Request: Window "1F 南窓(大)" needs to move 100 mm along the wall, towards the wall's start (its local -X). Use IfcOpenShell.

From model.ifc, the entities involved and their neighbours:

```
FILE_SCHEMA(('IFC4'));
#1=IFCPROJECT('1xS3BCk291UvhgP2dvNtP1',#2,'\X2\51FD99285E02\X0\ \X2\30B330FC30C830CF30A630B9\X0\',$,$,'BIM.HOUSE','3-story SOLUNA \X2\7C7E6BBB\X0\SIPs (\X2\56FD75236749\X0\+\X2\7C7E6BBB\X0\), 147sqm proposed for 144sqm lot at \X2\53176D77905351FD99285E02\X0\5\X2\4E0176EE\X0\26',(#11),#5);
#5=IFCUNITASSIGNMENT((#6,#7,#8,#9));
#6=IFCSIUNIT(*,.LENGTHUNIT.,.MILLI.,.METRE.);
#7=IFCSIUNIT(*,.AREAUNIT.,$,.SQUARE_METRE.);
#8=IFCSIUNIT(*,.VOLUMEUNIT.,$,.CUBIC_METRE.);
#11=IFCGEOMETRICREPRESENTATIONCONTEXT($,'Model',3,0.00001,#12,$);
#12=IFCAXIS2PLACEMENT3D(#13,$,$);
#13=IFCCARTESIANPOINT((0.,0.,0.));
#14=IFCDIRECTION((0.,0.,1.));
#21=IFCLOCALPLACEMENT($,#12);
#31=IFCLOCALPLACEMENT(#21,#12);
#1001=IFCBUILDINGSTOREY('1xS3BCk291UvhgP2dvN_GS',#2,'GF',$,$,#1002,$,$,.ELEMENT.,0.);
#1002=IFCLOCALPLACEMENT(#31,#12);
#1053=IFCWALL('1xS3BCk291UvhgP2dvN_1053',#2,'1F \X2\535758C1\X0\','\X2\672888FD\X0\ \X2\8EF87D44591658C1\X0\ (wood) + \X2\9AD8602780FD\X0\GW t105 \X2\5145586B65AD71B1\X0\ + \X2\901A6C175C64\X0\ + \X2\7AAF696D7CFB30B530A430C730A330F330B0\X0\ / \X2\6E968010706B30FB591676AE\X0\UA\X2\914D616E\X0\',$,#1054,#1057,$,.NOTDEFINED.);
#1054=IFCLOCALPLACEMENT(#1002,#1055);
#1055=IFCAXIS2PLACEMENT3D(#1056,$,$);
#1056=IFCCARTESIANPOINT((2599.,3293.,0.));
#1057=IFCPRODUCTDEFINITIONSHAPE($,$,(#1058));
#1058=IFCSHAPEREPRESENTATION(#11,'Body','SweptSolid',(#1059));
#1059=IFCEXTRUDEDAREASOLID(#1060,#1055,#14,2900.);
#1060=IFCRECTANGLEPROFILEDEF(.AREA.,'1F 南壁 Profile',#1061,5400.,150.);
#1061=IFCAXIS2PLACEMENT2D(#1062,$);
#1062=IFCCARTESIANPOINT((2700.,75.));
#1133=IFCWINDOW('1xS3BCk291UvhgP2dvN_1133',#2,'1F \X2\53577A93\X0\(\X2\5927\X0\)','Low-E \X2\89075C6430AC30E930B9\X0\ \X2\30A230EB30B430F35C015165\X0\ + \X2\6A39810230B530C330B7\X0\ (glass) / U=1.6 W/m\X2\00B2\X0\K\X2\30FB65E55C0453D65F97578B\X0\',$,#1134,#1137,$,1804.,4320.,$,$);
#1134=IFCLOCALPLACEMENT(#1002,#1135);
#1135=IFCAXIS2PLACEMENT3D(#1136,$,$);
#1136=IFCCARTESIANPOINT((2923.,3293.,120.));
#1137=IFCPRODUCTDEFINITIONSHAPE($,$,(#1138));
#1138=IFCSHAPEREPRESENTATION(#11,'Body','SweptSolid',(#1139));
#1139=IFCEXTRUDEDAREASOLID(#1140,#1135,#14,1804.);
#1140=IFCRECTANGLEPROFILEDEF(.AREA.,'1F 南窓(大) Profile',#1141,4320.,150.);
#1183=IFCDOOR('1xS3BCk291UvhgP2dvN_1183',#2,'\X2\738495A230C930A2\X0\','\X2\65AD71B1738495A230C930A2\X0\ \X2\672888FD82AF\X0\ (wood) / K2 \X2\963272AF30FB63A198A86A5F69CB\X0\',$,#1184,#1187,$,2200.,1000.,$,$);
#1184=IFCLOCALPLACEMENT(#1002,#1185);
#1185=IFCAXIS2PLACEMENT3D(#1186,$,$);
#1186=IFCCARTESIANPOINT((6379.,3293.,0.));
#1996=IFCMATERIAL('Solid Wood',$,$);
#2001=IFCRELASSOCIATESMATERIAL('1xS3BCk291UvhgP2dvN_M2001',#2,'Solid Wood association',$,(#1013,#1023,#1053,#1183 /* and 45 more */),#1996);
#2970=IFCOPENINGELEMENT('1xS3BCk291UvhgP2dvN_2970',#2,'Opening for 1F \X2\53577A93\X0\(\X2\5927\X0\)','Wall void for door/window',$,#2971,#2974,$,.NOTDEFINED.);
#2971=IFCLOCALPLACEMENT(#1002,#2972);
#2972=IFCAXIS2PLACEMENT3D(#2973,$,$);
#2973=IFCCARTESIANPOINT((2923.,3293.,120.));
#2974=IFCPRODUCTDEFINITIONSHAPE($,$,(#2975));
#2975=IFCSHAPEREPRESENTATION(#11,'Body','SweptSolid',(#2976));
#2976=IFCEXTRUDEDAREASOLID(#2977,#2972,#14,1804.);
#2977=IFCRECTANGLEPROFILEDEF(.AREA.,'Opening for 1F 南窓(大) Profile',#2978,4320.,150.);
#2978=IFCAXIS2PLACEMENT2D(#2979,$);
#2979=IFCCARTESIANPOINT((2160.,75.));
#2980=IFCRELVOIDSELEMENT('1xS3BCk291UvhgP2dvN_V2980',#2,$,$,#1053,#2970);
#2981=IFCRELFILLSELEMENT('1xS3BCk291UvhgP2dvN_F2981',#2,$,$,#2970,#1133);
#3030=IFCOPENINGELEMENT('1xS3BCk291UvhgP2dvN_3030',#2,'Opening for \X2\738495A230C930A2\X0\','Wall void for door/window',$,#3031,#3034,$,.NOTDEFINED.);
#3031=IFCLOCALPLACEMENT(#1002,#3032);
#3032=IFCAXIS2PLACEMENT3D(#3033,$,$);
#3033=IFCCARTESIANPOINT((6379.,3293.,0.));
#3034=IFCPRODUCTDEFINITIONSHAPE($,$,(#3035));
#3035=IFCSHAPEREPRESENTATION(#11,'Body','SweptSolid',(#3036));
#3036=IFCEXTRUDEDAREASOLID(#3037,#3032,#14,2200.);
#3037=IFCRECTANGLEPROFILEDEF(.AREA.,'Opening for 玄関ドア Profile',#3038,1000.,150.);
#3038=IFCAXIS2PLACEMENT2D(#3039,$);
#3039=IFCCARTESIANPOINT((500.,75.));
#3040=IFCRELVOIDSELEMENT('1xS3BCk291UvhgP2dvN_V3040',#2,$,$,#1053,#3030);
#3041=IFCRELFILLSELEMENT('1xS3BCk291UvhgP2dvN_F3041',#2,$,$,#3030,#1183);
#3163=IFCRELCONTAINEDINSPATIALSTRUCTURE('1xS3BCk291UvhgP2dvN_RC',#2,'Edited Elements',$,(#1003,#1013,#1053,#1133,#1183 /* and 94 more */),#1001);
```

```python
import ifcopenshell
import ifcopenshell.api.geometry
import ifcopenshell.util.placement
import ifcopenshell.util.unit

model = ifcopenshell.open("model.ifc")
unit_scale = ifcopenshell.util.unit.calculate_unit_scale(model)

window = model.by_guid("1xS3BCk291UvhgP2dvN_1133")
opening = window.FillsVoids[0].RelatingOpeningElement
wall = opening.VoidsElements[0].RelatingBuildingElement

wall_matrix = ifcopenshell.util.placement.get_local_placement(wall.ObjectPlacement)
shift = wall_matrix[:3, 0] * -0.1 / unit_scale
before = ifcopenshell.util.placement.get_local_placement(window.ObjectPlacement)[:3, 3].copy()

# The window is not placed relative to its opening, so move both.
for product in (opening, window):
    matrix = ifcopenshell.util.placement.get_local_placement(product.ObjectPlacement)
    matrix[:3, 3] += shift
    ifcopenshell.api.geometry.edit_object_placement(model, product=product, matrix=matrix, is_si=False)

after = ifcopenshell.util.placement.get_local_placement(window.ObjectPlacement)[:3, 3]
print("window moved by", (after - before).round(3) + 0.0)

model.write("model_edited.ifc")
```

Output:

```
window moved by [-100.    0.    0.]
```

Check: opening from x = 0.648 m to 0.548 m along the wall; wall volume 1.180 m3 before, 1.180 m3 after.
